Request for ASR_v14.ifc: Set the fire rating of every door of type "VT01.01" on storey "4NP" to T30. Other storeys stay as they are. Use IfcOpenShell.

First a look at what the model holds.

```python
import ifcopenshell
import ifcopenshell.util.element

model = ifcopenshell.open("ASR_v14.ifc")
print(model.schema)
storey = next(s for s in model.by_type("IfcBuildingStorey") if s.Name == "4NP")
doors = [e for e in ifcopenshell.util.element.get_decomposition(storey) if e.is_a("IfcDoor")]
seen = {}
for e in doors:
    element_type = ifcopenshell.util.element.get_type(e)
    key = (element_type.Name if element_type != e and element_type else None, ifcopenshell.util.element.get_pset(e, "Pset_DoorCommon", "FireRating"))
    seen[key] = seen.get(key, 0) + 1
for (name, value), count in sorted(seen.items(), key=str):
    print(count, "x", name, "|", value)
```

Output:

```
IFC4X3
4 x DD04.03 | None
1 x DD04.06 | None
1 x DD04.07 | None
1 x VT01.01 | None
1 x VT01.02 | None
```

```python
import ifcopenshell
import ifcopenshell.api.pset
import ifcopenshell.util.element

model = ifcopenshell.open("ASR_v14.ifc")

storey = next(s for s in model.by_type("IfcBuildingStorey") if s.Name == "4NP")
doors = [e for e in ifcopenshell.util.element.get_decomposition(storey) if e.is_a("IfcDoor")]

count = 0
for e in doors:
    element_type = ifcopenshell.util.element.get_type(e)
    if element_type in (None, e) or element_type.Name != "VT01.01":
        continue
    # add_pset returns the element's existing set when there is one.
    pset = ifcopenshell.api.pset.add_pset(model, product=e, name="Pset_DoorCommon")
    ifcopenshell.api.pset.edit_pset(model, pset=pset, properties={"FireRating": "T30"})
    count += 1

print(count, "doors updated")

model.write("ASR_v14_edited.ifc")
```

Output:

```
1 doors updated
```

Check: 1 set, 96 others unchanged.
